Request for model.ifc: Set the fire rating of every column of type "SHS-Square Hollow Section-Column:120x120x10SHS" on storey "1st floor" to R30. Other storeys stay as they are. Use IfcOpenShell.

First a look at what the model holds.

```python
import ifcopenshell
import ifcopenshell.util.element

model = ifcopenshell.open("model.ifc")
print(model.schema)
storey = next(s for s in model.by_type("IfcBuildingStorey") if s.Name == "1st floor")
columns = [e for e in ifcopenshell.util.element.get_decomposition(storey) if e.is_a("IfcColumn")]
seen = {}
for e in columns:
    element_type = ifcopenshell.util.element.get_type(e)
    key = (element_type.Name if element_type != e and element_type else None, ifcopenshell.util.element.get_pset(e, "Pset_ColumnCommon", "FireRating"))
    seen[key] = seen.get(key, 0) + 1
for (name, value), count in sorted(seen.items(), key=str):
    print(count, "x", name, "|", value)
```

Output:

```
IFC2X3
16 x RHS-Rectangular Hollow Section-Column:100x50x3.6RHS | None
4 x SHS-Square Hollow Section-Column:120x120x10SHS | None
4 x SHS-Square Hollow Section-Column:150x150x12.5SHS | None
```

```python
import ifcopenshell
import ifcopenshell.api.pset
import ifcopenshell.util.element

model = ifcopenshell.open("model.ifc")

storey = next(s for s in model.by_type("IfcBuildingStorey") if s.Name == "1st floor")
columns = [e for e in ifcopenshell.util.element.get_decomposition(storey) if e.is_a("IfcColumn")]

count = 0
for e in columns:
    element_type = ifcopenshell.util.element.get_type(e)
    if element_type in (None, e) or element_type.Name != "SHS-Square Hollow Section-Column:120x120x10SHS":
        continue
    # add_pset returns the element's existing set when there is one.
    pset = ifcopenshell.api.pset.add_pset(model, product=e, name="Pset_ColumnCommon")
    ifcopenshell.api.pset.edit_pset(model, pset=pset, properties={"FireRating": "R30"})
    count += 1

print(count, "columns updated")

model.write("model_v2.ifc")
```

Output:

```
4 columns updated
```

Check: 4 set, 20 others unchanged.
